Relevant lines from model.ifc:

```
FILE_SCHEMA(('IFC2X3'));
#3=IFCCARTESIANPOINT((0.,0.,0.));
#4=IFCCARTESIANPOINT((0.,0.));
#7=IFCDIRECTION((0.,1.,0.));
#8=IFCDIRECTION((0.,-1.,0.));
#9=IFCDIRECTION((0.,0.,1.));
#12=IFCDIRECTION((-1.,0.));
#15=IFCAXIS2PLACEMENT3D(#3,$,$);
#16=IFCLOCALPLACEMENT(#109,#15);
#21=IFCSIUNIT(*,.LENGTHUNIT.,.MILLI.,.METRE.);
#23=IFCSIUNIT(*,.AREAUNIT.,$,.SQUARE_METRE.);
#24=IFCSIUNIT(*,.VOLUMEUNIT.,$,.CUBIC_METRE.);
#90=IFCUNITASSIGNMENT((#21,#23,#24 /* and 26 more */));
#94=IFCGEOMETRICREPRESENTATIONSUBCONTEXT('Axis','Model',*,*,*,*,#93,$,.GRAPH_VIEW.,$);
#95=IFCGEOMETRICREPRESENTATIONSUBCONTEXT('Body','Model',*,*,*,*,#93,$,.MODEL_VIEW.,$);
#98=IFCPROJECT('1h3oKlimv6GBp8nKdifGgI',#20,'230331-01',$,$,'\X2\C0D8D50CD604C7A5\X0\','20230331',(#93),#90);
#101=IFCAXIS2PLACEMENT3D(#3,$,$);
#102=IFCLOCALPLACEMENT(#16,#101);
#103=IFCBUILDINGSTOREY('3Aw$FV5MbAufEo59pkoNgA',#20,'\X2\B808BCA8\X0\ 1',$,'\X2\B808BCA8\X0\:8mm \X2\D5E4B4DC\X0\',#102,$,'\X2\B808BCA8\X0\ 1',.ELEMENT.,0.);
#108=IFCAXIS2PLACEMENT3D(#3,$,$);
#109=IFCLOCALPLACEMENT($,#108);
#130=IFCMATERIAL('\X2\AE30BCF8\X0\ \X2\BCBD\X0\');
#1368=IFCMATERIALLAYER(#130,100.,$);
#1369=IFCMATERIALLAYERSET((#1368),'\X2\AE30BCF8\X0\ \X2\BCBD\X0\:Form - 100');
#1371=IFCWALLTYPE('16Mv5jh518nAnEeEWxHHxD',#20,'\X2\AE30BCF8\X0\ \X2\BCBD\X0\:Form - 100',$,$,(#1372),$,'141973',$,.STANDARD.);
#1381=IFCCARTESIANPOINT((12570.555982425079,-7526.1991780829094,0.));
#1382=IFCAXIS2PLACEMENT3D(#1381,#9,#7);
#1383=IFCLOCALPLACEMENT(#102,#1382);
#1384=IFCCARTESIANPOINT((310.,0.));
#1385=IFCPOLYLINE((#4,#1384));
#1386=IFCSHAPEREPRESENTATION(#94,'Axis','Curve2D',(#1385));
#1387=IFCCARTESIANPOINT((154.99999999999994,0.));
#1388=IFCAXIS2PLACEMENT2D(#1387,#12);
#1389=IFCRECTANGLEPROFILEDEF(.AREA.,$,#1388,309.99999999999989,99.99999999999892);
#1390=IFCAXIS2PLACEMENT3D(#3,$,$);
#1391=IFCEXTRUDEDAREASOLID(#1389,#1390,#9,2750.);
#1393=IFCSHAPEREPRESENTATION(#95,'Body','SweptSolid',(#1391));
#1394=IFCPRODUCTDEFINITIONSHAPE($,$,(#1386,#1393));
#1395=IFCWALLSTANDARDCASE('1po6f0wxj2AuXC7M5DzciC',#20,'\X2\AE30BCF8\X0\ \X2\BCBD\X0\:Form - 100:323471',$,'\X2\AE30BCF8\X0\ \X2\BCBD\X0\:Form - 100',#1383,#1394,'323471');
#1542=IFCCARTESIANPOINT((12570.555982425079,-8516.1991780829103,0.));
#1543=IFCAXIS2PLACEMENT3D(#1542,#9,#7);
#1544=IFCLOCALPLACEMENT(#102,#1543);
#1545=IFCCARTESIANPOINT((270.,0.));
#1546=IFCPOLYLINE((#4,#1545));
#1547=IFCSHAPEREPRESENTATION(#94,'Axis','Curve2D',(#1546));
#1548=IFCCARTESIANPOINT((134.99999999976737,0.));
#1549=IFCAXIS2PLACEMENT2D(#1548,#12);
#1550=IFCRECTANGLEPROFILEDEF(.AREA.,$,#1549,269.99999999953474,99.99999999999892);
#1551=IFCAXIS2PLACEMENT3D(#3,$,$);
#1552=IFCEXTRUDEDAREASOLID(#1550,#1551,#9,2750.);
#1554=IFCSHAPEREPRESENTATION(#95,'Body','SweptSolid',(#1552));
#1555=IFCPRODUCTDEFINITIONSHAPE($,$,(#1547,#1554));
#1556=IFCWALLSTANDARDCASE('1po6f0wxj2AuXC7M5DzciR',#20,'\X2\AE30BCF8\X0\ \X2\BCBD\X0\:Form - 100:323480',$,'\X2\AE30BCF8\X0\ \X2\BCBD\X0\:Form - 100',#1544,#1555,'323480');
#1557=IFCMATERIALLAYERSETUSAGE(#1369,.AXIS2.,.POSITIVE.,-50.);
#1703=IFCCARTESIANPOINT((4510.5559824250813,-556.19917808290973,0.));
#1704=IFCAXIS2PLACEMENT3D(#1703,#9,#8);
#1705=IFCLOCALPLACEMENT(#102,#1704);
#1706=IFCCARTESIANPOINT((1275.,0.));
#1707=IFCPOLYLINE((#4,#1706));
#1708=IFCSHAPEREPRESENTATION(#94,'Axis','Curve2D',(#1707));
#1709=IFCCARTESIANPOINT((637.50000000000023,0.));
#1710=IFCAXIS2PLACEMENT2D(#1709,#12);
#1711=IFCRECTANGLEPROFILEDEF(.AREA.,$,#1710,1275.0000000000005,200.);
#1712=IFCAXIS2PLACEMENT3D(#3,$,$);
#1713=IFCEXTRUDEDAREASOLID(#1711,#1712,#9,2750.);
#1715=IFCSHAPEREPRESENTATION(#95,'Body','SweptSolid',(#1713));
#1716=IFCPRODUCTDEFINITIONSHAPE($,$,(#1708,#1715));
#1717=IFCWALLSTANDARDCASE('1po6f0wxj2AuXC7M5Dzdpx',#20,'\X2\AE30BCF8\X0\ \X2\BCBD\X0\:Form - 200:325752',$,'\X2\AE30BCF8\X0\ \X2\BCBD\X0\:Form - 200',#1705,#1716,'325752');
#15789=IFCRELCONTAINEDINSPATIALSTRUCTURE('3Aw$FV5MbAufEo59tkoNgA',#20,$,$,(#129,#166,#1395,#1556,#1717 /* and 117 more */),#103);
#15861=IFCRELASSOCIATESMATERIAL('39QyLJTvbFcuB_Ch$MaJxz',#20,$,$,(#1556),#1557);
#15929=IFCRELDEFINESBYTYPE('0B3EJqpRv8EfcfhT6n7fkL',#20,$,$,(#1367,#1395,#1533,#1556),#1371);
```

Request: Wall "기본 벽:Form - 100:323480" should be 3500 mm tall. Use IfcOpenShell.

```python
import ifcopenshell
import ifcopenshell.geom
import ifcopenshell.util.representation
import ifcopenshell.util.shape
import ifcopenshell.util.unit

model = ifcopenshell.open("model.ifc")
unit_scale = ifcopenshell.util.unit.calculate_unit_scale(model)
settings = ifcopenshell.geom.settings()


def volume(element):
    """Net volume in cubic metres, openings subtracted."""
    shape = ifcopenshell.geom.create_shape(settings, element)
    return ifcopenshell.util.shape.get_volume(shape.geometry)


wall = model.by_guid("1po6f0wxj2AuXC7M5DzciR")
before = volume(wall)

body = ifcopenshell.util.representation.get_representation(wall, "Model", "Body")
solid = body.Items[0]
old_height = solid.Depth
solid.Depth = 3.5 / unit_scale
after = volume(wall)

print(f"height {old_height:g} -> {solid.Depth:g}, volume {before:.3f} -> {after:.3f} m3")

model.write("model_edited.ifc")
```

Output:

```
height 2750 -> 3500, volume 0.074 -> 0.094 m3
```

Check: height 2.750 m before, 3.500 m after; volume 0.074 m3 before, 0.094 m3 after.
